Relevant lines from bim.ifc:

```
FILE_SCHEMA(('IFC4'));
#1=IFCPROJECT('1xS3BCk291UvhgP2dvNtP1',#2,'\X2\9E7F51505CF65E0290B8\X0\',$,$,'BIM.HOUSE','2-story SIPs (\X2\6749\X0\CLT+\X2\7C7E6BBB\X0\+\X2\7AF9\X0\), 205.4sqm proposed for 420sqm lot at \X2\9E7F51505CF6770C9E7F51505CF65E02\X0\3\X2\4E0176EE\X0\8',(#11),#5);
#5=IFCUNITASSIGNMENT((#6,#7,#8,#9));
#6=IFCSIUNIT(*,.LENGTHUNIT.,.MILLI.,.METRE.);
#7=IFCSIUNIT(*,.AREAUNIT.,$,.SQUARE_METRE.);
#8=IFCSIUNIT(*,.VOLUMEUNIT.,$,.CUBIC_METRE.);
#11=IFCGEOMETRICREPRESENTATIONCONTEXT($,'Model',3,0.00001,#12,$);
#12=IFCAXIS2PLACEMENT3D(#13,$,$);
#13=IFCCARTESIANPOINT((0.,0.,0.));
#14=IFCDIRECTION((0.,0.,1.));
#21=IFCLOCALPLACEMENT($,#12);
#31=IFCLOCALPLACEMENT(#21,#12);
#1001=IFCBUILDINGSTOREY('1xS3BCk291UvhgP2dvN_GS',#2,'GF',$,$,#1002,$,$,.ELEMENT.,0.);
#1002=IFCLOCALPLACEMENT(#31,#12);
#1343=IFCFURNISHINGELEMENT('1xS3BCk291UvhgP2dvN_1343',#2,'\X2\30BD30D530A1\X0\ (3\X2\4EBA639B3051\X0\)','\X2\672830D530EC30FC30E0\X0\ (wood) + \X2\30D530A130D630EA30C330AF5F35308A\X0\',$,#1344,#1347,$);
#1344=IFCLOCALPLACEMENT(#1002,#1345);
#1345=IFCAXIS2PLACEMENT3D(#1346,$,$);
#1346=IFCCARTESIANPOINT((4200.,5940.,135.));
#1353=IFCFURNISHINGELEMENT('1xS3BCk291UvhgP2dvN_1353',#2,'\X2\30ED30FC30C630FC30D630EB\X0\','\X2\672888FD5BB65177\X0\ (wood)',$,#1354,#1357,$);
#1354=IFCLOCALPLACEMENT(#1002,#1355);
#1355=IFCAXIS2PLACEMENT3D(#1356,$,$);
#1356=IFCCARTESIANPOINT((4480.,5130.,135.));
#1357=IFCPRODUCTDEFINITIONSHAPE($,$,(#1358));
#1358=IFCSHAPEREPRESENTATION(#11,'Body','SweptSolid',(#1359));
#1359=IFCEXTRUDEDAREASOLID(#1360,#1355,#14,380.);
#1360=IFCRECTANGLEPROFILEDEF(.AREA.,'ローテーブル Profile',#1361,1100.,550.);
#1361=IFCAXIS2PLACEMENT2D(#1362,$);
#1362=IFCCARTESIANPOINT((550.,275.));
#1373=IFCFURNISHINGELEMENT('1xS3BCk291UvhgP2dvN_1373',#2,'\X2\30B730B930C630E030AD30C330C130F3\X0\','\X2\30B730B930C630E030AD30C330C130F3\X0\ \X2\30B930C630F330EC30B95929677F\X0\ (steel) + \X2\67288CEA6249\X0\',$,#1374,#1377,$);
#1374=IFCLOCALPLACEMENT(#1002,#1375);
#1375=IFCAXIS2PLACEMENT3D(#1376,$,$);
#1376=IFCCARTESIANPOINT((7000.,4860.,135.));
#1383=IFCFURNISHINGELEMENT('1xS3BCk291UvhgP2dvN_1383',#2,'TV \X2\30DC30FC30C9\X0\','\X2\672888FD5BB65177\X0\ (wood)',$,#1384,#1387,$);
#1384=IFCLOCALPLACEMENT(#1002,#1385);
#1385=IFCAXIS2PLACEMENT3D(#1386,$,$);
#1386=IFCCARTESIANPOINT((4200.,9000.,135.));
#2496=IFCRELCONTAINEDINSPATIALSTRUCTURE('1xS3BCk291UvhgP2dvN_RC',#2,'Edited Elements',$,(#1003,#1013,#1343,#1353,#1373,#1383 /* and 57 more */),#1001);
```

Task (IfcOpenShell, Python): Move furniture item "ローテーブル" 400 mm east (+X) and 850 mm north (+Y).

```python
import ifcopenshell
import ifcopenshell.api.geometry
import ifcopenshell.util.placement
import ifcopenshell.util.unit

model = ifcopenshell.open("bim.ifc")
unit_scale = ifcopenshell.util.unit.calculate_unit_scale(model)

item = model.by_id(1353)
matrix = ifcopenshell.util.placement.get_local_placement(item.ObjectPlacement)
matrix[0, 3] += 0.4 / unit_scale
matrix[1, 3] += 0.85 / unit_scale
ifcopenshell.api.geometry.edit_object_placement(model, product=item, matrix=matrix, is_si=False)

print(ifcopenshell.util.placement.get_local_placement(item.ObjectPlacement).round(3) + 0.0)

model.write("bim_v2.ifc")
```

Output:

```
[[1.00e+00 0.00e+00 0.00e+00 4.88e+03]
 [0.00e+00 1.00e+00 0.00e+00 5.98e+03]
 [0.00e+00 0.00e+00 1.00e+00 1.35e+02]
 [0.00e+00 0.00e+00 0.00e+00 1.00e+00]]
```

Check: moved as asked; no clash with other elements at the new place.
